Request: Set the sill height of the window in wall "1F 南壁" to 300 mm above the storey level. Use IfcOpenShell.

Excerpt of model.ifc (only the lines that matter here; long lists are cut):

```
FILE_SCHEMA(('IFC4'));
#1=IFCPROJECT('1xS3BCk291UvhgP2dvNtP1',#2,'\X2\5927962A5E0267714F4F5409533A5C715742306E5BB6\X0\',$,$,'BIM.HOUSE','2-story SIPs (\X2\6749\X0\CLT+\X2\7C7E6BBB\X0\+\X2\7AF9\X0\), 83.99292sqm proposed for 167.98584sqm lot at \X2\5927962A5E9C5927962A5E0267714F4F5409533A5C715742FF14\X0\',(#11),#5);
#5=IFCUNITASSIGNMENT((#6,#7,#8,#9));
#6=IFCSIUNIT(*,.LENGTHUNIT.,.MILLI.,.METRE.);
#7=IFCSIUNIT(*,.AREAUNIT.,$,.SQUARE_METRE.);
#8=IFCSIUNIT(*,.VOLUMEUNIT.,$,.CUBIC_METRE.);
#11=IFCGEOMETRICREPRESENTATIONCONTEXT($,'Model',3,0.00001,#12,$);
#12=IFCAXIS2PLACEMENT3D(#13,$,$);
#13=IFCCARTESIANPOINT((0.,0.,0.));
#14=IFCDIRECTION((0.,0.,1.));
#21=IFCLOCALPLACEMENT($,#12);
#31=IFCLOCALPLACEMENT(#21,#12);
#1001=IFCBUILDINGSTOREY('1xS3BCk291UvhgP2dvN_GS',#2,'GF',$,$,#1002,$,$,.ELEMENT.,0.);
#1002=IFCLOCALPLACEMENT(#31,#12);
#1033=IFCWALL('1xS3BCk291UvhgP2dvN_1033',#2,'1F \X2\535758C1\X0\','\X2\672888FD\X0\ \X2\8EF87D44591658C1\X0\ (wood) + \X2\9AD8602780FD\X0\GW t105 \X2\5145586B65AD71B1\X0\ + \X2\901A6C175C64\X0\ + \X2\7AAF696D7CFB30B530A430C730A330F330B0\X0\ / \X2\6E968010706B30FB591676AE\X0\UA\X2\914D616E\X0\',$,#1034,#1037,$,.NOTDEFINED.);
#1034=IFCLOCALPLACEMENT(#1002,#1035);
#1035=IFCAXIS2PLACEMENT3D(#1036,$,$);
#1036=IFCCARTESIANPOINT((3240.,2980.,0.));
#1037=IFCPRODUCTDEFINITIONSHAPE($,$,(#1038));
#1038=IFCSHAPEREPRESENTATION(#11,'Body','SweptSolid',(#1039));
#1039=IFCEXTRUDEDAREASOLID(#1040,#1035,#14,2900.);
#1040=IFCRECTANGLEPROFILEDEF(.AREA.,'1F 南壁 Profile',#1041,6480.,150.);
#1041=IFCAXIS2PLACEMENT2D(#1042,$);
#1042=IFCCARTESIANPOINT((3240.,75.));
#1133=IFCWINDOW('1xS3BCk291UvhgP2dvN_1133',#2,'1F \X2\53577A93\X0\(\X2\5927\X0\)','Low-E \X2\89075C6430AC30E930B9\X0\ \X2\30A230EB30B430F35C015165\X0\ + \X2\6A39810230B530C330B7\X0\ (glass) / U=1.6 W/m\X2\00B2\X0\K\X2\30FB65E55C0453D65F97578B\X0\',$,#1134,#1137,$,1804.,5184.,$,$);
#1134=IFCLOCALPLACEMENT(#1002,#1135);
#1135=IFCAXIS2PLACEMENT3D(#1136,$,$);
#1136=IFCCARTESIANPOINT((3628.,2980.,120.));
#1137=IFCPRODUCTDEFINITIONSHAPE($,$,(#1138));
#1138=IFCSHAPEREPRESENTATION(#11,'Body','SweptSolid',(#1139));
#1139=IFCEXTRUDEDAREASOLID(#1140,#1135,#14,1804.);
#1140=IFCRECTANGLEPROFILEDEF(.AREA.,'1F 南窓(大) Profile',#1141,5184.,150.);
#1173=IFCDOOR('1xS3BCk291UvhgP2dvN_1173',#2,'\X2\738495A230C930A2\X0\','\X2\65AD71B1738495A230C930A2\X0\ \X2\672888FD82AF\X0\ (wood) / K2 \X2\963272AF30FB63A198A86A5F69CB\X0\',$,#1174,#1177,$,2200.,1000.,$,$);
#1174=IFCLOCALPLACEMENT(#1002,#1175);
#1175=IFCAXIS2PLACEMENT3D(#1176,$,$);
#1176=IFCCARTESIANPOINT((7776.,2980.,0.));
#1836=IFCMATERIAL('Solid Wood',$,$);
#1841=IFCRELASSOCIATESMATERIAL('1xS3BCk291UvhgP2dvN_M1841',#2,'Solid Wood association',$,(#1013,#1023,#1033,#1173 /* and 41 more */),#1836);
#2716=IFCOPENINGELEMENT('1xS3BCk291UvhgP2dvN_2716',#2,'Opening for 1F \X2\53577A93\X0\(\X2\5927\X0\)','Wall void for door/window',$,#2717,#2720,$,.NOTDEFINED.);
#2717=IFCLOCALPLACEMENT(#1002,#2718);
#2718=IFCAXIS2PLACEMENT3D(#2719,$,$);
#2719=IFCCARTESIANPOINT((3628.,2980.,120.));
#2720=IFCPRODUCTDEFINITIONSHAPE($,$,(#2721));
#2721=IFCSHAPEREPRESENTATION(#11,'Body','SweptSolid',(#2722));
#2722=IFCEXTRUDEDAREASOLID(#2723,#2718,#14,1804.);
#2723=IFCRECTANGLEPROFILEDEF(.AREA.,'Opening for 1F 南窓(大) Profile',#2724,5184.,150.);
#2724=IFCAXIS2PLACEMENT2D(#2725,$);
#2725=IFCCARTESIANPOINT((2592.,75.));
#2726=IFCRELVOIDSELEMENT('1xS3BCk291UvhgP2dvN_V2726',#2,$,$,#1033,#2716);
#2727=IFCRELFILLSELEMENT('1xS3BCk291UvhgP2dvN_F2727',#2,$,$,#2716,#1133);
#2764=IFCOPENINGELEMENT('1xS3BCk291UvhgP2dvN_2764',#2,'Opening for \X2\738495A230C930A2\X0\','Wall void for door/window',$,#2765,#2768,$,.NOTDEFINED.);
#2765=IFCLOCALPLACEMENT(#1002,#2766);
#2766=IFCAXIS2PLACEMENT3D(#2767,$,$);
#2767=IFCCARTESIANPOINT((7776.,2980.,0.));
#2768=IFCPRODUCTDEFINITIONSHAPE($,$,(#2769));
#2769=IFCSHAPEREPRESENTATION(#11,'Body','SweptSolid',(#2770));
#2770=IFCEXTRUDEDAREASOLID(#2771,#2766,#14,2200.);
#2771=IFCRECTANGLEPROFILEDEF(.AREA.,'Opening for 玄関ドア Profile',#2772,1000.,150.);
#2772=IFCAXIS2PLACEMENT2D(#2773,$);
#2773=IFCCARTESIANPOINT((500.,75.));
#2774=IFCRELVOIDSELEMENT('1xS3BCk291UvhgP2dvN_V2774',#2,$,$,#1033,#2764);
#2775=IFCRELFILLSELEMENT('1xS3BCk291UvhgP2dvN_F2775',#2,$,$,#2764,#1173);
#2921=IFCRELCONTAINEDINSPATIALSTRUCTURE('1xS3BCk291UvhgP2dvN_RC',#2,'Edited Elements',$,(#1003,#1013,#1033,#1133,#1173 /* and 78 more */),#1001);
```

```python
import numpy as np
import ifcopenshell
import ifcopenshell.api.geometry
import ifcopenshell.geom
import ifcopenshell.util.element
import ifcopenshell.util.placement
import ifcopenshell.util.shape
import ifcopenshell.util.unit

model = ifcopenshell.open("model.ifc")
unit_scale = ifcopenshell.util.unit.calculate_unit_scale(model)

window = model.by_guid("1xS3BCk291UvhgP2dvN_1133")
opening = window.FillsVoids[0].RelatingOpeningElement
storey = ifcopenshell.util.element.get_container(window, ifc_class="IfcBuildingStorey")
level = ifcopenshell.util.placement.get_local_placement(storey.ObjectPlacement)[2, 3]

# The opening's origin need not be at the sill, so measure its lowest point.
shape = ifcopenshell.geom.create_shape(ifcopenshell.geom.settings(), opening)
bottom = ifcopenshell.util.shape.get_shape_bottom_elevation(shape, shape.geometry) / unit_scale
dz = level + 0.3 / unit_scale - bottom

shift = np.array([0.0, 0.0, dz])
# The window is not placed relative to its opening, so move both.
for product in (opening, window):
    matrix = ifcopenshell.util.placement.get_local_placement(product.ObjectPlacement)
    matrix[:3, 3] += shift
    ifcopenshell.api.geometry.edit_object_placement(model, product=product, matrix=matrix, is_si=False)

print(f"moved by {dz * unit_scale:+.3f} m")

model.write("model_rev.ifc")
```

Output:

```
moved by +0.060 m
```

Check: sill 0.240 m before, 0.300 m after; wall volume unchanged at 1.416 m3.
